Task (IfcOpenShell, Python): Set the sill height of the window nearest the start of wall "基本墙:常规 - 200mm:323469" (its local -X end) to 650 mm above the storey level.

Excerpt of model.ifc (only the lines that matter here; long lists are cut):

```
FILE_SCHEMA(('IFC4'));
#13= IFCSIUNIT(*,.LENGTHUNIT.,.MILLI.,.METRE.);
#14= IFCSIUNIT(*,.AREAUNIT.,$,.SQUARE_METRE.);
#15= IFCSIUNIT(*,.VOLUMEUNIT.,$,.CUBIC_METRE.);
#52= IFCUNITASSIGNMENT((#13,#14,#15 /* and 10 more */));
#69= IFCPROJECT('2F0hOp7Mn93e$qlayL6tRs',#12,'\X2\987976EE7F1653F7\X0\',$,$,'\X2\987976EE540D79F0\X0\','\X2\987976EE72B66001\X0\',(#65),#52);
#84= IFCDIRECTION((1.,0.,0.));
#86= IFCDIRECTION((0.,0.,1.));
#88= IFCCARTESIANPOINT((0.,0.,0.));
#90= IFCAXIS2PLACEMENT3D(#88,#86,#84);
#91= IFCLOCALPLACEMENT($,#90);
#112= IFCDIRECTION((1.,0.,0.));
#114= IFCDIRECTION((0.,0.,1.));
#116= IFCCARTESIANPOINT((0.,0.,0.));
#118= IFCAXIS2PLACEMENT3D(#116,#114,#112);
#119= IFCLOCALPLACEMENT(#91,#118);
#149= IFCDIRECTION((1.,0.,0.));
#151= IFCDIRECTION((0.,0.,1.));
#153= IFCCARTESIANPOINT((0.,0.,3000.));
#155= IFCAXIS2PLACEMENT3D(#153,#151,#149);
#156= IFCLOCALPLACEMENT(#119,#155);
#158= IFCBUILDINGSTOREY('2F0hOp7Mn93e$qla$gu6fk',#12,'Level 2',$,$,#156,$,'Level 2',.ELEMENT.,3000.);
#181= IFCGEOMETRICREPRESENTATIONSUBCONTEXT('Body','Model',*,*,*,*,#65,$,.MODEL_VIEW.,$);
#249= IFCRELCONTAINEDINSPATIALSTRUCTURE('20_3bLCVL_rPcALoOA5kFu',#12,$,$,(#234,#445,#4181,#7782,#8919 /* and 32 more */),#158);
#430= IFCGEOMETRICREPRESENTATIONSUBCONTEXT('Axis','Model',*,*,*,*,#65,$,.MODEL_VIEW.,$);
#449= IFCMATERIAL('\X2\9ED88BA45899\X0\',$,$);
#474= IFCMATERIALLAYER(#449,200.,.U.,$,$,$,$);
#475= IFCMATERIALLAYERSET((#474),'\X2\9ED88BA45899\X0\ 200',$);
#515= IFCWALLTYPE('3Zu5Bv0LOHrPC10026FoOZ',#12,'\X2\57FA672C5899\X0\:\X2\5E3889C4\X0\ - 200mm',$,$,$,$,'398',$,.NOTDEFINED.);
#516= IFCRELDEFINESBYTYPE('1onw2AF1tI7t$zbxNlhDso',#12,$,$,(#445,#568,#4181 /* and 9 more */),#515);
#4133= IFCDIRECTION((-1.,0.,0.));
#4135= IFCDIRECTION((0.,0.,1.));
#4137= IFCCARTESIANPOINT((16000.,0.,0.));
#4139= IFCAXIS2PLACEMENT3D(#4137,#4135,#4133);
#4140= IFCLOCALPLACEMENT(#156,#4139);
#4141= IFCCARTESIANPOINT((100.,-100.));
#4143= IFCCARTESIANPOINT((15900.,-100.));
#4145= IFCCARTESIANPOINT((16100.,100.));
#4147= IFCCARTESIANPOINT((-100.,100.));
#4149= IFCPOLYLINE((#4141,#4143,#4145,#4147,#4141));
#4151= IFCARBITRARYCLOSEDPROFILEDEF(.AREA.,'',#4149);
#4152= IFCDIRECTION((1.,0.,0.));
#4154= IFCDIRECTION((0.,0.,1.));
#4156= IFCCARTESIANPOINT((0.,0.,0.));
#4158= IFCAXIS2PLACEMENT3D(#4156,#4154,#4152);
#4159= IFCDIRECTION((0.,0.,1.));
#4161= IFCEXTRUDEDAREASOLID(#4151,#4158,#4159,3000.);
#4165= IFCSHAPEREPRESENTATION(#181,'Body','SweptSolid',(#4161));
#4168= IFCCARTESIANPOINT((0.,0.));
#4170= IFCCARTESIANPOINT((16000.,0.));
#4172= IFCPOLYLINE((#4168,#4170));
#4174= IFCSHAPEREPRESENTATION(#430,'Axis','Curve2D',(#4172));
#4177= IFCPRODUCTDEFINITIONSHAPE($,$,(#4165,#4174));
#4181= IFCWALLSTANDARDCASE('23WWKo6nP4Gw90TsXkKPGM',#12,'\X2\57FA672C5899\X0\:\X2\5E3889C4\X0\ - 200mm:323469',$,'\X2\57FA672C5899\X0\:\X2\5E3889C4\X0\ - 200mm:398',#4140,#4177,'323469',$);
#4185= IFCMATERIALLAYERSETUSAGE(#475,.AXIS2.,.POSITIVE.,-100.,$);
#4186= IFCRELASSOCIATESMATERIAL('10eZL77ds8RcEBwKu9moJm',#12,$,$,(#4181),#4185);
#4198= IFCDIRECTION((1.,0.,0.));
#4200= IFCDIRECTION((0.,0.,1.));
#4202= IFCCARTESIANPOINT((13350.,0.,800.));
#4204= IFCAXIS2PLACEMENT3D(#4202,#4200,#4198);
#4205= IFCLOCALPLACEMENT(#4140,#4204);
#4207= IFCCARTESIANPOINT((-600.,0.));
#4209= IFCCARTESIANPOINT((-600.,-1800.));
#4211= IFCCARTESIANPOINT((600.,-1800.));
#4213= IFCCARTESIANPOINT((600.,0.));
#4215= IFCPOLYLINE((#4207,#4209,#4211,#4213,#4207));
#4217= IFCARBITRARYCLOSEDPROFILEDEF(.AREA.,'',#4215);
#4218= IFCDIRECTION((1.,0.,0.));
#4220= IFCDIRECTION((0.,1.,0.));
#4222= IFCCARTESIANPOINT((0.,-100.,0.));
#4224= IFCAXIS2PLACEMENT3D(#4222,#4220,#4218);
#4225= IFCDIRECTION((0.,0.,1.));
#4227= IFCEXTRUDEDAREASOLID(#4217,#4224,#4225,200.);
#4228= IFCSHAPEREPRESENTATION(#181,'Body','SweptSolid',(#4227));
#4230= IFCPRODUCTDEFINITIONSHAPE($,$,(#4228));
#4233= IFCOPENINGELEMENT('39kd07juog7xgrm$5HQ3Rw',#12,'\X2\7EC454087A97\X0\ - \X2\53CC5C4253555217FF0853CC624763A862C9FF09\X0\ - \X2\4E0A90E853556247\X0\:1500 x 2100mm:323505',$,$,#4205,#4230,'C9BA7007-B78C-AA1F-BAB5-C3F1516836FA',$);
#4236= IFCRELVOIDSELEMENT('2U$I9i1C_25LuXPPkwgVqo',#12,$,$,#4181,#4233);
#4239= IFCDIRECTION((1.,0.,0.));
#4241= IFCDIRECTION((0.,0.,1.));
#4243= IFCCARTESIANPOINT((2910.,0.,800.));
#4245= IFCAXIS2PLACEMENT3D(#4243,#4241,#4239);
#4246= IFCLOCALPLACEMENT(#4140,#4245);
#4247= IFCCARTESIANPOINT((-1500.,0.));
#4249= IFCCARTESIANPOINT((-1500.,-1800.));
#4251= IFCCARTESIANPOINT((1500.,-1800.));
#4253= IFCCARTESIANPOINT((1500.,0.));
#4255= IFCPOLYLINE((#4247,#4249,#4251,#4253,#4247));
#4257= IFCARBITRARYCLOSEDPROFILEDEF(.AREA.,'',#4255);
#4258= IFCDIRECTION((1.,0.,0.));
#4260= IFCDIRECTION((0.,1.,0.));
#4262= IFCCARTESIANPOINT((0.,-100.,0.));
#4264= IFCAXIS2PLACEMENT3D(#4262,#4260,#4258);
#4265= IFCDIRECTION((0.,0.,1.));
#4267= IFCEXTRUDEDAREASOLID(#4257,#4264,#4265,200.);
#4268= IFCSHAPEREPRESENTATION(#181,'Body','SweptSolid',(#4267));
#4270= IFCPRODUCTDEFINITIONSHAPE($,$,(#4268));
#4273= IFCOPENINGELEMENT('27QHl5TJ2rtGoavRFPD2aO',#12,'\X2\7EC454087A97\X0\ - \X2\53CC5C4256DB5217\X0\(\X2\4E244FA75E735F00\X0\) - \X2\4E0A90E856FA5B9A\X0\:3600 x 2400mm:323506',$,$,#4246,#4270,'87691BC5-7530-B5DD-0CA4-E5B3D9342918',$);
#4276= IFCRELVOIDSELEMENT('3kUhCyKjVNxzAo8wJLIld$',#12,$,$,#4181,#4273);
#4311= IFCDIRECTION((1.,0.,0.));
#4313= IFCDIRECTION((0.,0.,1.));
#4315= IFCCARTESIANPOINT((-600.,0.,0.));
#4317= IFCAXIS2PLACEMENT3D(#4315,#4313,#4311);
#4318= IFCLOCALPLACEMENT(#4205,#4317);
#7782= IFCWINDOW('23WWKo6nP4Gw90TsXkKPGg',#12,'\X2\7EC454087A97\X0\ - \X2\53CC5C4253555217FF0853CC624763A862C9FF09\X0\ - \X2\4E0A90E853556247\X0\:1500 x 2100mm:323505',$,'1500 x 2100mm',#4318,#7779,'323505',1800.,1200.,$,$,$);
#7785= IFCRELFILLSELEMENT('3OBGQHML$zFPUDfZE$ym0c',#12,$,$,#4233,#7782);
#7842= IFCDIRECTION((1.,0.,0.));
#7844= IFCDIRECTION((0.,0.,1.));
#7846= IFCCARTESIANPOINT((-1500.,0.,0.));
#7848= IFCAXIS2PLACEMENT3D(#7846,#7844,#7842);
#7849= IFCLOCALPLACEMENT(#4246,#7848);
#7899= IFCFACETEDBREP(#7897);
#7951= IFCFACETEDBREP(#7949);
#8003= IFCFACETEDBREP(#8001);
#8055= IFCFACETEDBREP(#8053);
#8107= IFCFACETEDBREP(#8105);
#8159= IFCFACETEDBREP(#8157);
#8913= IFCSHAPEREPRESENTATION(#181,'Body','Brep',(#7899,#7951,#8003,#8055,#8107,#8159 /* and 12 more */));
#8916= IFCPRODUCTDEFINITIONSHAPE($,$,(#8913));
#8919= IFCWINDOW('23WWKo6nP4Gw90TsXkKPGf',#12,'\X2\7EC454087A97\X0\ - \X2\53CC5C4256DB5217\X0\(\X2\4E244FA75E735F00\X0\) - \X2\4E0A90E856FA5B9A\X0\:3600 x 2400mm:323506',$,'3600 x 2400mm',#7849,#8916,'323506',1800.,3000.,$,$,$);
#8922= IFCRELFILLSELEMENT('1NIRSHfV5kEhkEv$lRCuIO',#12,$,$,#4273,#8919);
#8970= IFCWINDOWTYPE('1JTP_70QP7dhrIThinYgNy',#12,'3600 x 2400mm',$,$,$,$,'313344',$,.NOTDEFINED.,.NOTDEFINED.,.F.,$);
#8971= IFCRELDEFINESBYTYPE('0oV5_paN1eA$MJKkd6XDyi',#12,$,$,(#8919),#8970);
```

```python
import numpy as np
import ifcopenshell
import ifcopenshell.api.geometry
import ifcopenshell.geom
import ifcopenshell.util.element
import ifcopenshell.util.placement
import ifcopenshell.util.shape
import ifcopenshell.util.unit

model = ifcopenshell.open("model.ifc")
unit_scale = ifcopenshell.util.unit.calculate_unit_scale(model)

window = model.by_id(8919)
opening = window.FillsVoids[0].RelatingOpeningElement
storey = ifcopenshell.util.element.get_container(window, ifc_class="IfcBuildingStorey")
level = ifcopenshell.util.placement.get_local_placement(storey.ObjectPlacement)[2, 3]

# The opening's origin need not be at the sill, so measure its lowest point.
shape = ifcopenshell.geom.create_shape(ifcopenshell.geom.settings(), opening)
bottom = ifcopenshell.util.shape.get_shape_bottom_elevation(shape, shape.geometry) / unit_scale
dz = level + 650.0 - bottom

shift = np.array([0.0, 0.0, dz])
# The window is placed relative to its opening, so it follows when the opening moves.
matrix = ifcopenshell.util.placement.get_local_placement(opening.ObjectPlacement)
matrix[:3, 3] += shift
ifcopenshell.api.geometry.edit_object_placement(
    model, product=opening, matrix=matrix, is_si=False, should_transform_children=True
)

print(f"moved by {dz * unit_scale:+.3f} m")

model.write("model_rev.ifc")
```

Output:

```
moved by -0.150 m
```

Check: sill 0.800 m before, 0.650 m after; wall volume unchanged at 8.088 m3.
